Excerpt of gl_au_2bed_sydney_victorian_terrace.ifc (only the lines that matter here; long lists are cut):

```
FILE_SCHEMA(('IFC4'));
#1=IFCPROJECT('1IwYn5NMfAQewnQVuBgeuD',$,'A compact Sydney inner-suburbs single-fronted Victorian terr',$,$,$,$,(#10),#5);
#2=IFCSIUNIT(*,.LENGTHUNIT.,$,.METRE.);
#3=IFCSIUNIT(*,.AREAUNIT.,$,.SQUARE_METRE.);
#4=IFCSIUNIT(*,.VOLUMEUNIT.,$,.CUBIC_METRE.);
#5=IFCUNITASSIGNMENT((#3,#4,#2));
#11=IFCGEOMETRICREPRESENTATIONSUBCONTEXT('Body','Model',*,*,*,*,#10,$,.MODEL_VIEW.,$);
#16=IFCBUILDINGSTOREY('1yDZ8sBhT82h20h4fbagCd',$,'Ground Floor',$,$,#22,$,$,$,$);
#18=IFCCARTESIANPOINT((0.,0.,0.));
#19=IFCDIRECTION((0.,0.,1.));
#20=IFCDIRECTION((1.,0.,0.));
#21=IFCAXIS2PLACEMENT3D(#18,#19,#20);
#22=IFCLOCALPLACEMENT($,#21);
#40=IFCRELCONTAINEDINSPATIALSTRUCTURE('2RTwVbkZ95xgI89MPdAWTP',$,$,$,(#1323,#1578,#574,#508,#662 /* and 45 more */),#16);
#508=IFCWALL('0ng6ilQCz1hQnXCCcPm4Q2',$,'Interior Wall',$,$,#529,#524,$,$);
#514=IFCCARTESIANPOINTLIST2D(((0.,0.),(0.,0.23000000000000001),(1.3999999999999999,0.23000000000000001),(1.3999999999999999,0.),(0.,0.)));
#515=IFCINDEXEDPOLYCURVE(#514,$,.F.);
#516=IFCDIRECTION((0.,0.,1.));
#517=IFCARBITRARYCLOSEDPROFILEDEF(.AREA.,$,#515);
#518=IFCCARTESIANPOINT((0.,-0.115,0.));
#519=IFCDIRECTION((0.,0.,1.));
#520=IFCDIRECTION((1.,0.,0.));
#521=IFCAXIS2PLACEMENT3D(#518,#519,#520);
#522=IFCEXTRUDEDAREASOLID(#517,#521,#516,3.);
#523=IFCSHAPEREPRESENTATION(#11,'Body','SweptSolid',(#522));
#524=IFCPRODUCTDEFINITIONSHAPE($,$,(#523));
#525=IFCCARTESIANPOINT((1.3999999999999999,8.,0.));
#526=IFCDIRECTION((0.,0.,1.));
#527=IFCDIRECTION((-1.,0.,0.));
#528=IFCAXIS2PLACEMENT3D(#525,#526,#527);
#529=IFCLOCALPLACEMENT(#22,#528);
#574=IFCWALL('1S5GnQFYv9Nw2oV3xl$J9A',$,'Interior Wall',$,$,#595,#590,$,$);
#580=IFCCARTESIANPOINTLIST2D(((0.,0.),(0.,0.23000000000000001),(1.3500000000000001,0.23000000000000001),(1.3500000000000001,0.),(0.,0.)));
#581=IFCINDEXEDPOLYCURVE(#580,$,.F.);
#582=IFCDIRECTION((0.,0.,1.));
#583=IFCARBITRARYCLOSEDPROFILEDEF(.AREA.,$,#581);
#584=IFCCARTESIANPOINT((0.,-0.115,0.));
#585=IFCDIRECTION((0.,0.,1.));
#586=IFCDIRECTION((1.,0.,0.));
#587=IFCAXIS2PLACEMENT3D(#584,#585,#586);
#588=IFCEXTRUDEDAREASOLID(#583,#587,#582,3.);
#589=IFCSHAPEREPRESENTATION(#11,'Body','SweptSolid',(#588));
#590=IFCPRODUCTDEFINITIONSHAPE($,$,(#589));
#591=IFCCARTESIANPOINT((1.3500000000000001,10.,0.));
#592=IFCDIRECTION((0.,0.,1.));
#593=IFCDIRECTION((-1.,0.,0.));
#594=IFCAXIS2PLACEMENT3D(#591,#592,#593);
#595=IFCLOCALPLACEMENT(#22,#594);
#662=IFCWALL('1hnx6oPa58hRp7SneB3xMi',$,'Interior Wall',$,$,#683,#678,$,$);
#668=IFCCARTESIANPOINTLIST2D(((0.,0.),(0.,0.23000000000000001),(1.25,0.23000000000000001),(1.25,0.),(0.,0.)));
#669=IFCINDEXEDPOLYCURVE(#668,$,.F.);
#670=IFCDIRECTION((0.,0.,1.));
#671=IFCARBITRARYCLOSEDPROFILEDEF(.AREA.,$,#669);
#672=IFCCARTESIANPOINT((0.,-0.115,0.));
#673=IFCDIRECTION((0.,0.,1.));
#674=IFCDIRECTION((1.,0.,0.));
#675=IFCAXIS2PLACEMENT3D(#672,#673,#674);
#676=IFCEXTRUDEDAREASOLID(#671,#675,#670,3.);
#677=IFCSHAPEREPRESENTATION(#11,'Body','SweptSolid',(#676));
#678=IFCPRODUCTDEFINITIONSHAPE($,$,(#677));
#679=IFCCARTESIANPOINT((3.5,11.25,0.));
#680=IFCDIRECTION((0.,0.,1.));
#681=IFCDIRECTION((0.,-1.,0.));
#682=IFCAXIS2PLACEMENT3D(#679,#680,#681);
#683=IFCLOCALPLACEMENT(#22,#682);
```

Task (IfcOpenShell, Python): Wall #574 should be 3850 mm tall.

```python
import ifcopenshell
import ifcopenshell.geom
import ifcopenshell.util.representation
import ifcopenshell.util.shape
import ifcopenshell.util.unit

model = ifcopenshell.open("gl_au_2bed_sydney_victorian_terrace.ifc")
unit_scale = ifcopenshell.util.unit.calculate_unit_scale(model)
settings = ifcopenshell.geom.settings()


def volume(element):
    """Net volume in cubic metres, openings subtracted."""
    shape = ifcopenshell.geom.create_shape(settings, element)
    return ifcopenshell.util.shape.get_volume(shape.geometry)


wall = model.by_guid("1S5GnQFYv9Nw2oV3xl$J9A")
before = volume(wall)

body = ifcopenshell.util.representation.get_representation(wall, "Model", "Body")
solid = body.Items[0]
old_height = solid.Depth
solid.Depth = 3.85 / unit_scale
after = volume(wall)

print(f"height {old_height:g} -> {solid.Depth:g}, volume {before:.3f} -> {after:.3f} m3")

model.write("gl_au_2bed_sydney_victorian_terrace_v2.ifc")
```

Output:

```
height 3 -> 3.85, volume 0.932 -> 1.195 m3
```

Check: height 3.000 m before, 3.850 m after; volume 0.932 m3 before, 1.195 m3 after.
